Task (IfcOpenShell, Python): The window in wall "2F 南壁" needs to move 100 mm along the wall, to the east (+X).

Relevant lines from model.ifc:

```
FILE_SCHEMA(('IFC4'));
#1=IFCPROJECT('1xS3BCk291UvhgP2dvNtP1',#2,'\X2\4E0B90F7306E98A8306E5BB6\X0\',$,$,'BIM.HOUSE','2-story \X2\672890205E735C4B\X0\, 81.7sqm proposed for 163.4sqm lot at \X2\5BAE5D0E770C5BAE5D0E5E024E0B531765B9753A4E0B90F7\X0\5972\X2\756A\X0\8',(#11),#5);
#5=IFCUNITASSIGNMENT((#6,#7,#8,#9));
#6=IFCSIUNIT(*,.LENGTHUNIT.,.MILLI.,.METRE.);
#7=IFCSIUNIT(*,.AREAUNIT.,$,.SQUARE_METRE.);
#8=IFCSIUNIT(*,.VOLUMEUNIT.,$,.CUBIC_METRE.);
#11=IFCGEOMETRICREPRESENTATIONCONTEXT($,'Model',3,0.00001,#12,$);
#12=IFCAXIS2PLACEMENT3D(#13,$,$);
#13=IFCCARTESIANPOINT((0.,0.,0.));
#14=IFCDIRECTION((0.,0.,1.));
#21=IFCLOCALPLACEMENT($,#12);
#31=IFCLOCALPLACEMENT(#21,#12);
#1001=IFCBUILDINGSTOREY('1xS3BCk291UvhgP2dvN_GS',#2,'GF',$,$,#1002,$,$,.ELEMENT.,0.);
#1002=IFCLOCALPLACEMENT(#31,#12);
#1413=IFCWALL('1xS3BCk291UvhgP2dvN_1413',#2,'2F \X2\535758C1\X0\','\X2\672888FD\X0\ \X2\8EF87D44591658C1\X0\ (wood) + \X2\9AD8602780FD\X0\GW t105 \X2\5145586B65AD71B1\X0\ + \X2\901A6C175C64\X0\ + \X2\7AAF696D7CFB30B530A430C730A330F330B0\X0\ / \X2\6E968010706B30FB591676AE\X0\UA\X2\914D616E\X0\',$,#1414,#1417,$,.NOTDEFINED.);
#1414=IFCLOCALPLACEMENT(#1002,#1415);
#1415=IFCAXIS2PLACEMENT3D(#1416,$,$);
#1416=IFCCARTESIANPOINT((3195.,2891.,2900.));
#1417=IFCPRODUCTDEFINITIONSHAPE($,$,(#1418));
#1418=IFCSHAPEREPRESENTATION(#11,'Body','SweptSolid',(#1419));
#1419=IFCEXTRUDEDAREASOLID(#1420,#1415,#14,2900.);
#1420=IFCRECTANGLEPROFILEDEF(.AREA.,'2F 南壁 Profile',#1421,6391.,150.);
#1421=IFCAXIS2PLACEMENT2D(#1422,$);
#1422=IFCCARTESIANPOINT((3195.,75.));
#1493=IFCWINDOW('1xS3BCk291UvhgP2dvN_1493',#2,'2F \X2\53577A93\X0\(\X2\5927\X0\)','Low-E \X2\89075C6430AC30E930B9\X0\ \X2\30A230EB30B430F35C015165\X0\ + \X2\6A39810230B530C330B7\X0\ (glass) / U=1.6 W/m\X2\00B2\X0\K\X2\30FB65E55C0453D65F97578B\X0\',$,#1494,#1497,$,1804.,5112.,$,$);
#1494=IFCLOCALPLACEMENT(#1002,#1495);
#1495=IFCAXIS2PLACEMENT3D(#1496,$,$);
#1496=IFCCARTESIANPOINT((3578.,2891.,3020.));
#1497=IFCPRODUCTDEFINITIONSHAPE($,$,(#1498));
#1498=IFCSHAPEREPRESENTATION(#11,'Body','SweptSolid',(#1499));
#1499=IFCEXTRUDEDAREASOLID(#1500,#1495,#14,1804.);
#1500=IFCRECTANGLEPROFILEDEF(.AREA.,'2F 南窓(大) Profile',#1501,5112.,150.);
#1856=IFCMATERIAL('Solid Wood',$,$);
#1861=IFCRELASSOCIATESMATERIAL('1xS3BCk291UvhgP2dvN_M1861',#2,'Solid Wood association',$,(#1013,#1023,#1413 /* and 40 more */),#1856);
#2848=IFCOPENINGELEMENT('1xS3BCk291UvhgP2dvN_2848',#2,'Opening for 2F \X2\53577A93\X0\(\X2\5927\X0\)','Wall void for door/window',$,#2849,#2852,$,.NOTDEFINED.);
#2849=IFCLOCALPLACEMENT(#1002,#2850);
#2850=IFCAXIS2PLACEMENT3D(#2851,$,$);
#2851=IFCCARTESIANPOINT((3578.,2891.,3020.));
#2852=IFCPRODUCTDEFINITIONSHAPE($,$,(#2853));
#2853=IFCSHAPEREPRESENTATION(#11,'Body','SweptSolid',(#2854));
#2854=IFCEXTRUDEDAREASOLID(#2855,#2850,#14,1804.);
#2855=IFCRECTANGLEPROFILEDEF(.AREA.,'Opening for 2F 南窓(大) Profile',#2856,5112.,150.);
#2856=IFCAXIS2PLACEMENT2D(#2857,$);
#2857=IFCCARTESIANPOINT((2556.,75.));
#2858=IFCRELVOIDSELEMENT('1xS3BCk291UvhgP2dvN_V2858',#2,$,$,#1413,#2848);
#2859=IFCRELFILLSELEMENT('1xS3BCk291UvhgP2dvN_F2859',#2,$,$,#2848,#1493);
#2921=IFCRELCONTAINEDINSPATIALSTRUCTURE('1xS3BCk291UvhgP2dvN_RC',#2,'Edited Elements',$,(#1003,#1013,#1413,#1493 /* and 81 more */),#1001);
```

```python
import ifcopenshell
import ifcopenshell.api.geometry
import ifcopenshell.util.placement

model = ifcopenshell.open("model.ifc")

window = model.by_guid("1xS3BCk291UvhgP2dvN_1493")
opening = window.FillsVoids[0].RelatingOpeningElement
wall = opening.VoidsElements[0].RelatingBuildingElement

wall_matrix = ifcopenshell.util.placement.get_local_placement(wall.ObjectPlacement)
shift = wall_matrix[:3, 0] * 100.0
before = ifcopenshell.util.placement.get_local_placement(window.ObjectPlacement)[:3, 3].copy()

# The window is not placed relative to its opening, so move both.
for product in (opening, window):
    matrix = ifcopenshell.util.placement.get_local_placement(product.ObjectPlacement)
    matrix[:3, 3] += shift
    ifcopenshell.api.geometry.edit_object_placement(model, product=product, matrix=matrix, is_si=False)

after = ifcopenshell.util.placement.get_local_placement(window.ObjectPlacement)[:3, 3]
print("window moved by", (after - before).round(3) + 0.0)

model.write("model_v2.ifc")
```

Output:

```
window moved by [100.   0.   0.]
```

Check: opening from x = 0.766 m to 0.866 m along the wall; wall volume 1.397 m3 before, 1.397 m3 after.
